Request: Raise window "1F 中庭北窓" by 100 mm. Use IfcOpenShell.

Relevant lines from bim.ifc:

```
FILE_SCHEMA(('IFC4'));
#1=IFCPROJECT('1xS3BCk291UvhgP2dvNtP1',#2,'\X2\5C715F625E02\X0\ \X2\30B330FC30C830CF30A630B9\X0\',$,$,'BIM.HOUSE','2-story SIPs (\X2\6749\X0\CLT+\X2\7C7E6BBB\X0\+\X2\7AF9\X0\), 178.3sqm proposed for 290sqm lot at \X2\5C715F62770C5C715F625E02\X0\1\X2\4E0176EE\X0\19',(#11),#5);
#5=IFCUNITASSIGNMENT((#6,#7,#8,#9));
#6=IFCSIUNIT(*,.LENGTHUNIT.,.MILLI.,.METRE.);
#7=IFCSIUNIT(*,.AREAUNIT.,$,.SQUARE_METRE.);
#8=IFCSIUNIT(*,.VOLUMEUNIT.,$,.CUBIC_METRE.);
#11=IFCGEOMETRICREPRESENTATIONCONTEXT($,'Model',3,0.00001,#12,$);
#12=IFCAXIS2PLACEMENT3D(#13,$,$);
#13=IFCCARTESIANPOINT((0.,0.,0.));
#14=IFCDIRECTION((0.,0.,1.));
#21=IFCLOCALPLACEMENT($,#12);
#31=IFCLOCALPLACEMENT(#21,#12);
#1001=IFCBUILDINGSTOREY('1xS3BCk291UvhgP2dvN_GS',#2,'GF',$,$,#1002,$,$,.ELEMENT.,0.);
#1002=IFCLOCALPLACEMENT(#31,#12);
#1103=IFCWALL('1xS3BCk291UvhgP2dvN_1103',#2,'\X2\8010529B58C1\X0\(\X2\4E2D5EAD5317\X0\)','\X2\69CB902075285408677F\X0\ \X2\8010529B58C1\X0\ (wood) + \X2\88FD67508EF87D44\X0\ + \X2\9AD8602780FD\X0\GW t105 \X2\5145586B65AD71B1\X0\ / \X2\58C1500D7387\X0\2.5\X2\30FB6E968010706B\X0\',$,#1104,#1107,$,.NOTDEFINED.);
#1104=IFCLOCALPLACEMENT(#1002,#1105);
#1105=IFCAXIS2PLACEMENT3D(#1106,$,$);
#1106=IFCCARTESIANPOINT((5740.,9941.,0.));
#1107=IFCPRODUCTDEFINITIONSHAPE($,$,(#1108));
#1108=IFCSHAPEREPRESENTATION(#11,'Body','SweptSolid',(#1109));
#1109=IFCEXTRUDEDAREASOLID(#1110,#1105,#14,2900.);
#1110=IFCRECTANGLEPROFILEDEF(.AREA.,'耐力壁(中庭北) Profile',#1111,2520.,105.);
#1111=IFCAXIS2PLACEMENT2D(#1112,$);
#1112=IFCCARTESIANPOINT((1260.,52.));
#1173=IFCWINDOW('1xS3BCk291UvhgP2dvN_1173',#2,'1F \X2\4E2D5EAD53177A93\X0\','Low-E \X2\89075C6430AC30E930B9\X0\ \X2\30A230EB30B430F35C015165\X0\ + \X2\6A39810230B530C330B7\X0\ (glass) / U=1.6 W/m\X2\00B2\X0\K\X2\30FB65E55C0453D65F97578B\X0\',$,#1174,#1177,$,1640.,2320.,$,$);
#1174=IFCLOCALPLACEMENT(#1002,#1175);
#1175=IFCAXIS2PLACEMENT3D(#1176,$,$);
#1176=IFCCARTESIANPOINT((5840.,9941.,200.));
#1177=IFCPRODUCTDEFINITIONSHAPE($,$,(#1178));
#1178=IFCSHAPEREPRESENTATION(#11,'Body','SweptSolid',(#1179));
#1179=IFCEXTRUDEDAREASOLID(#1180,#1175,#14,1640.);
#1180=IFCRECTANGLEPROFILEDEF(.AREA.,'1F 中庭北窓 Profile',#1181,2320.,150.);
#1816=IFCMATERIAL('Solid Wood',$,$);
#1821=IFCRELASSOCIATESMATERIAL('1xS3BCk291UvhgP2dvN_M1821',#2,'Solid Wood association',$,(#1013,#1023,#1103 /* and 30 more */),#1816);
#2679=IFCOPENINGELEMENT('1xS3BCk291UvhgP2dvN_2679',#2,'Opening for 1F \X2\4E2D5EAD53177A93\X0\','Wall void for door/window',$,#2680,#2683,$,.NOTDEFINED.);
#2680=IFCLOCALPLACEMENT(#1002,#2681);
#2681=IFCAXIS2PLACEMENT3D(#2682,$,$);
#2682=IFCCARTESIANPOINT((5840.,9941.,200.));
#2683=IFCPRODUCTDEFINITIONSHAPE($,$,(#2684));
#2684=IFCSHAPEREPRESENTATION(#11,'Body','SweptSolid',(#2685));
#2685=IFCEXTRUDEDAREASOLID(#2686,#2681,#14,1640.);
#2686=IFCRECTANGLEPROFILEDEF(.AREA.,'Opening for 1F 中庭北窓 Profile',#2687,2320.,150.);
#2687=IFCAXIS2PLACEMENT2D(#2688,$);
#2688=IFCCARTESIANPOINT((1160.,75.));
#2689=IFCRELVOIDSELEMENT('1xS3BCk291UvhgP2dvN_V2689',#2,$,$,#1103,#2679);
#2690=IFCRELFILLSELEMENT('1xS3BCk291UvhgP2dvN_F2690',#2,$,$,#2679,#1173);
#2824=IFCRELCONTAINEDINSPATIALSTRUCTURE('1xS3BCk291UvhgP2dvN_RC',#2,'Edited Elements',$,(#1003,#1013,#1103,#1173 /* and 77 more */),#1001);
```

```python
import numpy as np
import ifcopenshell
import ifcopenshell.api.geometry
import ifcopenshell.util.placement
import ifcopenshell.util.unit

model = ifcopenshell.open("bim.ifc")
unit_scale = ifcopenshell.util.unit.calculate_unit_scale(model)

window = model.by_guid("1xS3BCk291UvhgP2dvN_1173")
opening = window.FillsVoids[0].RelatingOpeningElement
dz = 0.1 / unit_scale

shift = np.array([0.0, 0.0, dz])
# The window is not placed relative to its opening, so move both.
for product in (opening, window):
    matrix = ifcopenshell.util.placement.get_local_placement(product.ObjectPlacement)
    matrix[:3, 3] += shift
    ifcopenshell.api.geometry.edit_object_placement(model, product=product, matrix=matrix, is_si=False)

print(f"moved by {dz * unit_scale:+.3f} m")

model.write("bim-out.ifc")
```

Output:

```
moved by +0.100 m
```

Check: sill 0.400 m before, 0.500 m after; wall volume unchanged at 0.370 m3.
